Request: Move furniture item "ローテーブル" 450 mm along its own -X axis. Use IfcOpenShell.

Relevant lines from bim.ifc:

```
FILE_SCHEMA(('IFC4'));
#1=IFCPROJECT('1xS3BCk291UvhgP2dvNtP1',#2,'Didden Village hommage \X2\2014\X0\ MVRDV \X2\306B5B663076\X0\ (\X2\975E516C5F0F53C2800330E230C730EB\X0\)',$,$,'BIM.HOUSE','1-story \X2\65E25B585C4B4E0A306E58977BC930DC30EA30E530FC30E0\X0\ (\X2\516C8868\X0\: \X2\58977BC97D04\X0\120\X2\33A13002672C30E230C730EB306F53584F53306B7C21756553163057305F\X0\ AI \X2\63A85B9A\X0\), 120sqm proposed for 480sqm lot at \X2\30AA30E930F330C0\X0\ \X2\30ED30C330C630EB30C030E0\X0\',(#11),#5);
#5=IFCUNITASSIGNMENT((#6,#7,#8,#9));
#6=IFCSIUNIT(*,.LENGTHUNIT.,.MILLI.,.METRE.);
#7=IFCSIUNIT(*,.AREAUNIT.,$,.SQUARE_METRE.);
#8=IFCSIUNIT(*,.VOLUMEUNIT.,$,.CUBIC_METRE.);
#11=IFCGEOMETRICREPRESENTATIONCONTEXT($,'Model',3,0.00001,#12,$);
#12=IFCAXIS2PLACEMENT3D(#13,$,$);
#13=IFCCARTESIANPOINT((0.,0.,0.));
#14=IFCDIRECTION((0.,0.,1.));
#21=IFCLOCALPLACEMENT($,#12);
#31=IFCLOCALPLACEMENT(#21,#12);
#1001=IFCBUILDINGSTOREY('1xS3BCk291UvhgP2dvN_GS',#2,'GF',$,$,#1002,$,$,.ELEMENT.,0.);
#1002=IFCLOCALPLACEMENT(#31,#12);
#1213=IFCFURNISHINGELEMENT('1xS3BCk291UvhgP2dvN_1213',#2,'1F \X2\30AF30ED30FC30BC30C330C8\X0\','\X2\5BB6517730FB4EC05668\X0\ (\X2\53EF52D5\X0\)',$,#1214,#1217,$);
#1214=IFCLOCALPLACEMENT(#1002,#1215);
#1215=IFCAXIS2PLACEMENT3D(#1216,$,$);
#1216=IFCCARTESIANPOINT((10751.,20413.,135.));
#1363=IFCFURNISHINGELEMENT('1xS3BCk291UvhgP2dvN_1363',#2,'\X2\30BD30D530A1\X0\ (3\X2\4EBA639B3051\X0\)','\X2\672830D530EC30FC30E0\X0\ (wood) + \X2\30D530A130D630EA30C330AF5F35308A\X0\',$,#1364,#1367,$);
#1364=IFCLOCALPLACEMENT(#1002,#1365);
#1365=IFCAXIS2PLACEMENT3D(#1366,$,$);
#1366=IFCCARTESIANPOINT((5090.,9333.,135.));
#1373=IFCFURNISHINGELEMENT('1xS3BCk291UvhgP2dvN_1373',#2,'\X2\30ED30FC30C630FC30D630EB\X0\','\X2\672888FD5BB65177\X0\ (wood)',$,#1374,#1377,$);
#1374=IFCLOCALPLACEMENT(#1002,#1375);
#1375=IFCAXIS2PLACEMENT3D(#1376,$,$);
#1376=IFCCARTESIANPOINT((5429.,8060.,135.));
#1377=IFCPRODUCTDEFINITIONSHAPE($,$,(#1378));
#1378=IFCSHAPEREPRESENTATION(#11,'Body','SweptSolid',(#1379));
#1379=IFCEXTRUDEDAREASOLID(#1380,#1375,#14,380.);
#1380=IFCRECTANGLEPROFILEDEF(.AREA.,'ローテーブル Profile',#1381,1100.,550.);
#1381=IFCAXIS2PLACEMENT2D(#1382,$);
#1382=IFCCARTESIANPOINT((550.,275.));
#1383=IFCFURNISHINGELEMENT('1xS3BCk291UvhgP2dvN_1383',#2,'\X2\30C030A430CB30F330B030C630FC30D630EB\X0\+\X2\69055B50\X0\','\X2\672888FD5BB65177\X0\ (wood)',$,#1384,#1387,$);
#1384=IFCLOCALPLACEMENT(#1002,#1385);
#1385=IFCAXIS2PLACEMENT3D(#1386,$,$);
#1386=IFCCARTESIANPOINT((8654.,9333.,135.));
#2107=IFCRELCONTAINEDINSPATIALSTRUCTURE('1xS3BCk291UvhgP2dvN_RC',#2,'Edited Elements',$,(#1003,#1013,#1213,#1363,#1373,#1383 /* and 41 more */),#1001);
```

```python
import ifcopenshell
import ifcopenshell.api.geometry
import ifcopenshell.util.placement
import ifcopenshell.util.unit

model = ifcopenshell.open("bim.ifc")
unit_scale = ifcopenshell.util.unit.calculate_unit_scale(model)

item = model.by_guid("1xS3BCk291UvhgP2dvN_1373")
matrix = ifcopenshell.util.placement.get_local_placement(item.ObjectPlacement)
matrix[:3, 3] -= matrix[:3, 0] * 0.45 / unit_scale
ifcopenshell.api.geometry.edit_object_placement(model, product=item, matrix=matrix, is_si=False)

print(ifcopenshell.util.placement.get_local_placement(item.ObjectPlacement).round(3) + 0.0)

model.write("bim_edited.ifc")
```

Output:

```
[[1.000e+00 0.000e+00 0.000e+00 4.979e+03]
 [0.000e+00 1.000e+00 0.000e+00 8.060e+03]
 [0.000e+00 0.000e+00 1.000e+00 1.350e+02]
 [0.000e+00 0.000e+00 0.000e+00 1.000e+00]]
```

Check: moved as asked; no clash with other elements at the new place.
